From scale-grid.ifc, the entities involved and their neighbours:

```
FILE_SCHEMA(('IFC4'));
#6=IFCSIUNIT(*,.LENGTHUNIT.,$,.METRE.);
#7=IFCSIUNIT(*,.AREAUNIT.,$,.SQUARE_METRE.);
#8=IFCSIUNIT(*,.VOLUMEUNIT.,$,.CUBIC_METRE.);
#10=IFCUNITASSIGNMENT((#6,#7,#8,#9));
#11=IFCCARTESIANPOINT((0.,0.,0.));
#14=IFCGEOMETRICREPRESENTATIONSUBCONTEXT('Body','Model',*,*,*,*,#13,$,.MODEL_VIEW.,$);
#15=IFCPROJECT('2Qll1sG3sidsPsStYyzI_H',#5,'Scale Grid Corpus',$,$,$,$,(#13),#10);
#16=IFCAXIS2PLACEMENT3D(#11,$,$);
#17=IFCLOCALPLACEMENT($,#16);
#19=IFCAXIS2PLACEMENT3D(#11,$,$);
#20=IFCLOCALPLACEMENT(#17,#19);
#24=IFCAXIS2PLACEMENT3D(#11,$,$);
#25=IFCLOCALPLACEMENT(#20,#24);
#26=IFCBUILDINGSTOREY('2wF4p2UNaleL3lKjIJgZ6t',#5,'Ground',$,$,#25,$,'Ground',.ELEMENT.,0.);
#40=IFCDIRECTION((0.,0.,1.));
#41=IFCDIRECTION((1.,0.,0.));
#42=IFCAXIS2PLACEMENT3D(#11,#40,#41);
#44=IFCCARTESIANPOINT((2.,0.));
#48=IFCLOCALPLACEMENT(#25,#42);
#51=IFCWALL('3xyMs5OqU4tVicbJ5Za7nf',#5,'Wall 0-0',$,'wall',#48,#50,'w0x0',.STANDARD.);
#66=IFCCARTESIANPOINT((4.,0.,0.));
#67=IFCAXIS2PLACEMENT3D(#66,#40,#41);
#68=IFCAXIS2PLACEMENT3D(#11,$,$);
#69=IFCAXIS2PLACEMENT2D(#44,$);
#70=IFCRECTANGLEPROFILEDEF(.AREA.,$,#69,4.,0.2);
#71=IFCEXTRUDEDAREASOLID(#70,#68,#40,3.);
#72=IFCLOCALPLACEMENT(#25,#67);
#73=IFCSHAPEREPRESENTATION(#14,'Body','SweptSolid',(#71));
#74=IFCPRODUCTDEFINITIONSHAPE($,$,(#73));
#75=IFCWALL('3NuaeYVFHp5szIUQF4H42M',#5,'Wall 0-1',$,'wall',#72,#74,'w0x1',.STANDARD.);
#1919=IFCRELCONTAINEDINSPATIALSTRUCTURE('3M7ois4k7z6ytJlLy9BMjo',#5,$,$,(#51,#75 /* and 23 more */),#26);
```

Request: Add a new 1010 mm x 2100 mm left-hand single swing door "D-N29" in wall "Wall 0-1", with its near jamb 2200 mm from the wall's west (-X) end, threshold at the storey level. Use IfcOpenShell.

```python
import numpy as np
import ifcopenshell
import ifcopenshell.api.feature
import ifcopenshell.api.geometry
import ifcopenshell.api.root
import ifcopenshell.api.spatial
import ifcopenshell.geom
import ifcopenshell.util.element
import ifcopenshell.util.placement
import ifcopenshell.util.representation
import ifcopenshell.util.shape
import ifcopenshell.util.unit

model = ifcopenshell.open("scale-grid.ifc")
unit_scale = ifcopenshell.util.unit.calculate_unit_scale(model)
settings = ifcopenshell.geom.settings()


def volume(element):
    """Net volume in cubic metres, openings subtracted."""
    shape = ifcopenshell.geom.create_shape(settings, element)
    return ifcopenshell.util.shape.get_volume(shape.geometry)


wall = model.by_id(75)
storey = ifcopenshell.util.element.get_container(wall, ifc_class="IfcBuildingStorey")
context = ifcopenshell.util.representation.get_context(model, "Model", "Body", "MODEL_VIEW")
before = volume(wall)

width, height, from_end, sill = 1.01, 2.1, 2.2, 0.0  # metres

# The wall runs along its own X axis, and the end named is its -X end.
wall_shape = ifcopenshell.geom.create_shape(settings, wall)
x, y, z = ifcopenshell.util.shape.get_vertices(wall_shape.geometry).T
start = x.min() + from_end
face, thickness = float(y.min()), float(y.max() - y.min())
wall_matrix = ifcopenshell.util.placement.get_local_placement(wall.ObjectPlacement)
level = ifcopenshell.util.placement.get_local_placement(storey.ObjectPlacement)[2, 3]


def in_wall(x, y):
    """Placement at x, y metres in the wall's axes, at sill height."""
    matrix = wall_matrix.copy()
    matrix[:, 3] = wall_matrix @ np.array([x / unit_scale, y / unit_scale, 0.0, 1.0])
    matrix[2, 3] = level + sill / unit_scale
    return matrix


# Opening: a box that overshoots both wall faces by 50 mm.
opening = ifcopenshell.api.root.create_entity(model, ifc_class="IfcOpeningElement", predefined_type="OPENING")
box = ifcopenshell.api.geometry.add_wall_representation(
    model, context=context, length=width, height=height, thickness=thickness + 0.1
)
ifcopenshell.api.geometry.assign_representation(model, product=opening, representation=box)
ifcopenshell.api.geometry.edit_object_placement(model, product=opening, matrix=in_wall(start, face - 0.05), is_si=False)
ifcopenshell.api.feature.add_feature(model, feature=opening, element=wall)

door = ifcopenshell.api.root.create_entity(model, ifc_class="IfcDoor", name="D-N29", predefined_type="DOOR")
door.OverallWidth, door.OverallHeight = width / unit_scale, height / unit_scale
door.OperationType = "SINGLE_SWING_LEFT"
body = ifcopenshell.api.geometry.add_door_representation(
    model,
    context=context,
    overall_width=door.OverallWidth,
    overall_height=door.OverallHeight,
    operation_type="SINGLE_SWING_LEFT",
    lining_properties={"LiningDepth": thickness / unit_scale, "ThresholdDepth": thickness / unit_scale},
)
ifcopenshell.api.geometry.assign_representation(model, product=door, representation=body)
ifcopenshell.api.spatial.assign_container(model, products=[door], relating_structure=storey)
ifcopenshell.api.feature.add_filling(model, opening=opening, element=door)

# The lining spans the wall, so the door starts at the wall face.
ifcopenshell.api.geometry.edit_object_placement(model, product=door, matrix=in_wall(start, face), is_si=False)

after = volume(wall)

print(f"wall volume {before:.3f} -> {after:.3f} m3")

model.write("scale-grid_rev.ifc")
```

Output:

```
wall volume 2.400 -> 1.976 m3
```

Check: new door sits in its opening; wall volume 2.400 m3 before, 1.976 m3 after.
